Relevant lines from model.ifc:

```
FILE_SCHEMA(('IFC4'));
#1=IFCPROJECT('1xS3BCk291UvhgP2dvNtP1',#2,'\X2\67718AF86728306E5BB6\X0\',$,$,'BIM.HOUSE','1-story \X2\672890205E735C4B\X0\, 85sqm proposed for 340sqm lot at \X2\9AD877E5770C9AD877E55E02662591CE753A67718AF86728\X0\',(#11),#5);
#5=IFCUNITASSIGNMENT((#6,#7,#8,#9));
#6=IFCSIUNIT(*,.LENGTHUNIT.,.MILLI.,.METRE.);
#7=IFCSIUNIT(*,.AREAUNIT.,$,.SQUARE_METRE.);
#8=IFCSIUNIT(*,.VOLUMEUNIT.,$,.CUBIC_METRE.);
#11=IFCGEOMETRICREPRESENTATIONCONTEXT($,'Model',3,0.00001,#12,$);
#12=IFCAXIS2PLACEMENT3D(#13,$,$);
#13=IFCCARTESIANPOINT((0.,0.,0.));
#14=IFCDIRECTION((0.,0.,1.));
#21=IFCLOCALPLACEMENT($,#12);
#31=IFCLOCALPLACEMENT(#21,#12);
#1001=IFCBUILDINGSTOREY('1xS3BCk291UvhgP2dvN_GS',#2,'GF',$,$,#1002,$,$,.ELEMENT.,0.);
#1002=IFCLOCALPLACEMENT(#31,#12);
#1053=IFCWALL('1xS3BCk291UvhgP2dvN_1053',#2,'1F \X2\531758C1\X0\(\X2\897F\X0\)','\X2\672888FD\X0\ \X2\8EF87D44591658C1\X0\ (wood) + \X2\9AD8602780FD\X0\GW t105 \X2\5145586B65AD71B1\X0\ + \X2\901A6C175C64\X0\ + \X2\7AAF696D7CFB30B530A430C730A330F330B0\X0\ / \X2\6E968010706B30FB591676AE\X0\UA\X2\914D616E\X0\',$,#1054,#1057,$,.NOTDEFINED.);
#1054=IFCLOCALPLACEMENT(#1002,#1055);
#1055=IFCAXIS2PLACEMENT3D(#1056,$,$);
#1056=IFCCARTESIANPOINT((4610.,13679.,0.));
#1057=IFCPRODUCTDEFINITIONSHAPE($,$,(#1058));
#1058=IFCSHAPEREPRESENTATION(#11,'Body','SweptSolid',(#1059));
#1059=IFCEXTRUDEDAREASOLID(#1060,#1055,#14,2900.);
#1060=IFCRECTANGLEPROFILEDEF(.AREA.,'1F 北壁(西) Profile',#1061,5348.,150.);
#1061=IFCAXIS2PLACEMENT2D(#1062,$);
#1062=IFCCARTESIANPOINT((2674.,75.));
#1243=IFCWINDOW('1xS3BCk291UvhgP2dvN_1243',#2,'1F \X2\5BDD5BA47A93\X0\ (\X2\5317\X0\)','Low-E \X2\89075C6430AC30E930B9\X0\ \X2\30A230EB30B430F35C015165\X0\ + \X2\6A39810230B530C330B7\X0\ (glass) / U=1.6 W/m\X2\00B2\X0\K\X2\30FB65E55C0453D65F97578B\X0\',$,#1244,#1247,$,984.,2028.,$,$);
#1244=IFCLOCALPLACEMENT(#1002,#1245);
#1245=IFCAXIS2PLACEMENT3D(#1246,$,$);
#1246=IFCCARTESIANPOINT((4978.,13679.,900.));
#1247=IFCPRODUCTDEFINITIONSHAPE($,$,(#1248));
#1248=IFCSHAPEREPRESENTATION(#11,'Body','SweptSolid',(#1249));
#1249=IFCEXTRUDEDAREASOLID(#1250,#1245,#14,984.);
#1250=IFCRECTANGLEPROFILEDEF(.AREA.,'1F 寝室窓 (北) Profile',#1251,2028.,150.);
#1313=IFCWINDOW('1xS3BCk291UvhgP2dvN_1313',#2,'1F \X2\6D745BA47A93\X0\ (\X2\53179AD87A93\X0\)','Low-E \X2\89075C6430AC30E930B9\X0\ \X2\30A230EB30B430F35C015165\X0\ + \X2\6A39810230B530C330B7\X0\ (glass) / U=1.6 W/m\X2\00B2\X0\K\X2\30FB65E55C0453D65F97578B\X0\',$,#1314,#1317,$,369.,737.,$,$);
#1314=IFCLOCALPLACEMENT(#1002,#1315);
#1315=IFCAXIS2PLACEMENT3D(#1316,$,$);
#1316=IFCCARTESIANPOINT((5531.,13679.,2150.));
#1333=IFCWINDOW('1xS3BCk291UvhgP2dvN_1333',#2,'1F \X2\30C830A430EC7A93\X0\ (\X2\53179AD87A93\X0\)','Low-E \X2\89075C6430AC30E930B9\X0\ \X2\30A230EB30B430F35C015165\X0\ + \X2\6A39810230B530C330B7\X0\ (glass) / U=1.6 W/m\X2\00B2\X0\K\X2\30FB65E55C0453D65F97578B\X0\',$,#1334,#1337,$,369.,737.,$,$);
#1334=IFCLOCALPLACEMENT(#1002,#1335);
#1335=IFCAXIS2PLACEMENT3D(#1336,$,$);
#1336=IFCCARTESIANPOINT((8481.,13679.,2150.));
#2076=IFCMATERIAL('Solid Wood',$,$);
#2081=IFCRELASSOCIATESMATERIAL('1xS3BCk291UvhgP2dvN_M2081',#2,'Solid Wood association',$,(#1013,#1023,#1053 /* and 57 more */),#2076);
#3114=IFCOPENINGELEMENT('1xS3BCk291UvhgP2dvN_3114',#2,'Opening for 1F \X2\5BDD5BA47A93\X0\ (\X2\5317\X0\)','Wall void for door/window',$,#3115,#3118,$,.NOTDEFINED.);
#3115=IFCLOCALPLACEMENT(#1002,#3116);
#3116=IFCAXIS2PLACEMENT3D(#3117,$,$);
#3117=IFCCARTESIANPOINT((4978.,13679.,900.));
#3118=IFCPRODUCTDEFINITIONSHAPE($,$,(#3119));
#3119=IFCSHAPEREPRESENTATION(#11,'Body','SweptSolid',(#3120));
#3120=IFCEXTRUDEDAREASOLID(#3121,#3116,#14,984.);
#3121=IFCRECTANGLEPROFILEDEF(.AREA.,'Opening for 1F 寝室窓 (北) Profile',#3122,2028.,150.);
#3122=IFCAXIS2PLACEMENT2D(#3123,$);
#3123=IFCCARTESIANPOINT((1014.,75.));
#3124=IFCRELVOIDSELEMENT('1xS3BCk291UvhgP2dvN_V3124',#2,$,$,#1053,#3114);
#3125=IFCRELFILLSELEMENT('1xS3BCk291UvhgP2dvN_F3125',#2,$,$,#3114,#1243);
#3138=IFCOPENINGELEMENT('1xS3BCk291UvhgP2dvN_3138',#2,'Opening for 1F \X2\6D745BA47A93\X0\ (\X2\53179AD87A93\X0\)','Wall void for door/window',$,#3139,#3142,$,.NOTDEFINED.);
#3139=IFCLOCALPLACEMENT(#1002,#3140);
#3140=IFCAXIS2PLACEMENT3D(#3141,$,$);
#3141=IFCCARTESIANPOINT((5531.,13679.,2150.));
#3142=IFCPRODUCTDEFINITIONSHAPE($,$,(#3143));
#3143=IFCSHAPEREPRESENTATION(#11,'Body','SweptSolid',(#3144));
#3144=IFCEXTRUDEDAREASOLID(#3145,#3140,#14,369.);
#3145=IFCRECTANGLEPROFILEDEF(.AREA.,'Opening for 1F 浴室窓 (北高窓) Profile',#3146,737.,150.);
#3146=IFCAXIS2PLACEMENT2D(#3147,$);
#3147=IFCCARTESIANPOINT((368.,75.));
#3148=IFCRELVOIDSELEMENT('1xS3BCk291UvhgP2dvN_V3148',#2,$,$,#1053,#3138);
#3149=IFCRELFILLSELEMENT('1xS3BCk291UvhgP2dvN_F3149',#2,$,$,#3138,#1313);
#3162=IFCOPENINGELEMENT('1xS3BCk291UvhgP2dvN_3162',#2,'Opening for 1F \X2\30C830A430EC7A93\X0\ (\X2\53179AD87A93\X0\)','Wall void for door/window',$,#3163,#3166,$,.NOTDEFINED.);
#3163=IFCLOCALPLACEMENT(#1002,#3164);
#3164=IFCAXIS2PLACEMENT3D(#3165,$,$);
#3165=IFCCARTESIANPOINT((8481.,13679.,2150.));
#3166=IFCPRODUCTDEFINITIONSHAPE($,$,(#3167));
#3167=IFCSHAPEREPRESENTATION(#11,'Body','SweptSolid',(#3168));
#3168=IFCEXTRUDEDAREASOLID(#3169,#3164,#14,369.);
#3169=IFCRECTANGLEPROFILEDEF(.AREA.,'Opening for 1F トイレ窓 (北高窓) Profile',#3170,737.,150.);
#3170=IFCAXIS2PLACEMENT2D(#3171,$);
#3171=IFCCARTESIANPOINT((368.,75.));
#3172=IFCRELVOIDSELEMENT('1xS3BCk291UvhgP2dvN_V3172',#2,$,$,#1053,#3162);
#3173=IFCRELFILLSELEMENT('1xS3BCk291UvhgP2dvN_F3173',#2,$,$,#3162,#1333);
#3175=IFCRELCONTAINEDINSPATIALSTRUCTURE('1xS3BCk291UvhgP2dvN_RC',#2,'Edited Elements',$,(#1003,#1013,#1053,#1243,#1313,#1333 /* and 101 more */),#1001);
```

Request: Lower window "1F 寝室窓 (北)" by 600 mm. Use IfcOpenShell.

```python
import numpy as np
import ifcopenshell
import ifcopenshell.api.geometry
import ifcopenshell.util.placement
import ifcopenshell.util.unit

model = ifcopenshell.open("model.ifc")
unit_scale = ifcopenshell.util.unit.calculate_unit_scale(model)

window = model.by_guid("1xS3BCk291UvhgP2dvN_1243")
opening = window.FillsVoids[0].RelatingOpeningElement
dz = -0.6 / unit_scale

shift = np.array([0.0, 0.0, dz])
# The window is not placed relative to its opening, so move both.
for product in (opening, window):
    matrix = ifcopenshell.util.placement.get_local_placement(product.ObjectPlacement)
    matrix[:3, 3] += shift
    ifcopenshell.api.geometry.edit_object_placement(model, product=product, matrix=matrix, is_si=False)

print(f"moved by {dz * unit_scale:+.3f} m")

model.write("model_edited.ifc")
```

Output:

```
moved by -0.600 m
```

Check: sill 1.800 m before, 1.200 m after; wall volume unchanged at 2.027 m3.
